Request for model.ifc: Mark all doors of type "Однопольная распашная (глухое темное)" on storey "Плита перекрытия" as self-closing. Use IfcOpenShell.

First a look at what the model holds.

```python
import ifcopenshell
import ifcopenshell.util.element

model = ifcopenshell.open("model.ifc")
print(model.schema)
storey = next(s for s in model.by_type("IfcBuildingStorey") if s.Name == "Плита перекрытия")
doors = [e for e in ifcopenshell.util.element.get_decomposition(storey) if e.is_a("IfcDoor")]
seen = {}
for e in doors:
    element_type = ifcopenshell.util.element.get_type(e)
    key = (element_type.Name if element_type != e and element_type else None, ifcopenshell.util.element.get_pset(e, "Pset_DoorCommon", "SelfClosing"))
    seen[key] = seen.get(key, 0) + 1
for (name, value), count in sorted(seen.items(), key=str):
    print(count, "x", name, "|", value)
```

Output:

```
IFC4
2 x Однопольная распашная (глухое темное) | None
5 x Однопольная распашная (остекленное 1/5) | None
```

```python
import ifcopenshell
import ifcopenshell.api.pset
import ifcopenshell.util.element

model = ifcopenshell.open("model.ifc")

storey = next(s for s in model.by_type("IfcBuildingStorey") if s.Name == "Плита перекрытия")
doors = [e for e in ifcopenshell.util.element.get_decomposition(storey) if e.is_a("IfcDoor")]

count = 0
for e in doors:
    element_type = ifcopenshell.util.element.get_type(e)
    if element_type in (None, e) or element_type.Name != "Однопольная распашная (глухое темное)":
        continue
    # add_pset returns the element's existing set when there is one.
    pset = ifcopenshell.api.pset.add_pset(model, product=e, name="Pset_DoorCommon")
    ifcopenshell.api.pset.edit_pset(model, pset=pset, properties={"SelfClosing": True})
    count += 1

print(count, "doors updated")

model.write("model_updated.ifc")
```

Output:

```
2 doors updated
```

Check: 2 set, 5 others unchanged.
